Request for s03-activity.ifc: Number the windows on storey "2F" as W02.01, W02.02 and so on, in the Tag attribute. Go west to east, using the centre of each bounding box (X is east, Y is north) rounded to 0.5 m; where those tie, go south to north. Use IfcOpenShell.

First a look at what the model holds.

```python
import ifcopenshell
import ifcopenshell.util.element
import ifcopenshell.util.placement

model = ifcopenshell.open("s03-activity.ifc")
print(model.schema)
storey = next(s for s in model.by_type("IfcBuildingStorey") if s.Name == "2F")
windows = [e for e in ifcopenshell.util.element.get_decomposition(storey) if e.is_a("IfcWindow")]
for e in sorted(windows, key=lambda e: e.id()):
    origin = ifcopenshell.util.placement.get_local_placement(e.ObjectPlacement)[:3, 3]
    print(e.id(), e.Tag, e.Name, origin.round(2) + 0.0, sep=" | ")
```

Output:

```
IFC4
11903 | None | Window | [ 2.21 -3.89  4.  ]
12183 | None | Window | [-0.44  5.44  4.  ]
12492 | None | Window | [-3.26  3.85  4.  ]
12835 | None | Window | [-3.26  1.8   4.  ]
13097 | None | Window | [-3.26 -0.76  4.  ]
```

```python
import ifcopenshell
import ifcopenshell.geom
import ifcopenshell.util.element
import ifcopenshell.util.shape

model = ifcopenshell.open("s03-activity.ifc")
settings = ifcopenshell.geom.settings()
settings.set("use-world-coords", True)


def centre(element):
    shape = ifcopenshell.geom.create_shape(settings, element)
    return ifcopenshell.util.shape.get_bbox_centroid(shape.geometry)


storey = next(s for s in model.by_type("IfcBuildingStorey") if s.Name == "2F")
windows = [e for e in ifcopenshell.util.element.get_decomposition(storey) if e.is_a("IfcWindow")]

# Insertion points can sit at a corner or the storey origin, so sort by the geometry (in metres).
centres = {e: centre(e) for e in windows}
windows.sort(key=lambda e: (round(centres[e][0] / 0.5), centres[e][1]))

for i, e in enumerate(windows, start=1):
    number = f"W02.{i:02d}"
    e.Tag = number
    print(e.id(), number)

model.write("s03-activity_updated.ifc")
```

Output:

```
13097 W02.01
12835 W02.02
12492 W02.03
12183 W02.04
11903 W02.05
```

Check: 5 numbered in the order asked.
